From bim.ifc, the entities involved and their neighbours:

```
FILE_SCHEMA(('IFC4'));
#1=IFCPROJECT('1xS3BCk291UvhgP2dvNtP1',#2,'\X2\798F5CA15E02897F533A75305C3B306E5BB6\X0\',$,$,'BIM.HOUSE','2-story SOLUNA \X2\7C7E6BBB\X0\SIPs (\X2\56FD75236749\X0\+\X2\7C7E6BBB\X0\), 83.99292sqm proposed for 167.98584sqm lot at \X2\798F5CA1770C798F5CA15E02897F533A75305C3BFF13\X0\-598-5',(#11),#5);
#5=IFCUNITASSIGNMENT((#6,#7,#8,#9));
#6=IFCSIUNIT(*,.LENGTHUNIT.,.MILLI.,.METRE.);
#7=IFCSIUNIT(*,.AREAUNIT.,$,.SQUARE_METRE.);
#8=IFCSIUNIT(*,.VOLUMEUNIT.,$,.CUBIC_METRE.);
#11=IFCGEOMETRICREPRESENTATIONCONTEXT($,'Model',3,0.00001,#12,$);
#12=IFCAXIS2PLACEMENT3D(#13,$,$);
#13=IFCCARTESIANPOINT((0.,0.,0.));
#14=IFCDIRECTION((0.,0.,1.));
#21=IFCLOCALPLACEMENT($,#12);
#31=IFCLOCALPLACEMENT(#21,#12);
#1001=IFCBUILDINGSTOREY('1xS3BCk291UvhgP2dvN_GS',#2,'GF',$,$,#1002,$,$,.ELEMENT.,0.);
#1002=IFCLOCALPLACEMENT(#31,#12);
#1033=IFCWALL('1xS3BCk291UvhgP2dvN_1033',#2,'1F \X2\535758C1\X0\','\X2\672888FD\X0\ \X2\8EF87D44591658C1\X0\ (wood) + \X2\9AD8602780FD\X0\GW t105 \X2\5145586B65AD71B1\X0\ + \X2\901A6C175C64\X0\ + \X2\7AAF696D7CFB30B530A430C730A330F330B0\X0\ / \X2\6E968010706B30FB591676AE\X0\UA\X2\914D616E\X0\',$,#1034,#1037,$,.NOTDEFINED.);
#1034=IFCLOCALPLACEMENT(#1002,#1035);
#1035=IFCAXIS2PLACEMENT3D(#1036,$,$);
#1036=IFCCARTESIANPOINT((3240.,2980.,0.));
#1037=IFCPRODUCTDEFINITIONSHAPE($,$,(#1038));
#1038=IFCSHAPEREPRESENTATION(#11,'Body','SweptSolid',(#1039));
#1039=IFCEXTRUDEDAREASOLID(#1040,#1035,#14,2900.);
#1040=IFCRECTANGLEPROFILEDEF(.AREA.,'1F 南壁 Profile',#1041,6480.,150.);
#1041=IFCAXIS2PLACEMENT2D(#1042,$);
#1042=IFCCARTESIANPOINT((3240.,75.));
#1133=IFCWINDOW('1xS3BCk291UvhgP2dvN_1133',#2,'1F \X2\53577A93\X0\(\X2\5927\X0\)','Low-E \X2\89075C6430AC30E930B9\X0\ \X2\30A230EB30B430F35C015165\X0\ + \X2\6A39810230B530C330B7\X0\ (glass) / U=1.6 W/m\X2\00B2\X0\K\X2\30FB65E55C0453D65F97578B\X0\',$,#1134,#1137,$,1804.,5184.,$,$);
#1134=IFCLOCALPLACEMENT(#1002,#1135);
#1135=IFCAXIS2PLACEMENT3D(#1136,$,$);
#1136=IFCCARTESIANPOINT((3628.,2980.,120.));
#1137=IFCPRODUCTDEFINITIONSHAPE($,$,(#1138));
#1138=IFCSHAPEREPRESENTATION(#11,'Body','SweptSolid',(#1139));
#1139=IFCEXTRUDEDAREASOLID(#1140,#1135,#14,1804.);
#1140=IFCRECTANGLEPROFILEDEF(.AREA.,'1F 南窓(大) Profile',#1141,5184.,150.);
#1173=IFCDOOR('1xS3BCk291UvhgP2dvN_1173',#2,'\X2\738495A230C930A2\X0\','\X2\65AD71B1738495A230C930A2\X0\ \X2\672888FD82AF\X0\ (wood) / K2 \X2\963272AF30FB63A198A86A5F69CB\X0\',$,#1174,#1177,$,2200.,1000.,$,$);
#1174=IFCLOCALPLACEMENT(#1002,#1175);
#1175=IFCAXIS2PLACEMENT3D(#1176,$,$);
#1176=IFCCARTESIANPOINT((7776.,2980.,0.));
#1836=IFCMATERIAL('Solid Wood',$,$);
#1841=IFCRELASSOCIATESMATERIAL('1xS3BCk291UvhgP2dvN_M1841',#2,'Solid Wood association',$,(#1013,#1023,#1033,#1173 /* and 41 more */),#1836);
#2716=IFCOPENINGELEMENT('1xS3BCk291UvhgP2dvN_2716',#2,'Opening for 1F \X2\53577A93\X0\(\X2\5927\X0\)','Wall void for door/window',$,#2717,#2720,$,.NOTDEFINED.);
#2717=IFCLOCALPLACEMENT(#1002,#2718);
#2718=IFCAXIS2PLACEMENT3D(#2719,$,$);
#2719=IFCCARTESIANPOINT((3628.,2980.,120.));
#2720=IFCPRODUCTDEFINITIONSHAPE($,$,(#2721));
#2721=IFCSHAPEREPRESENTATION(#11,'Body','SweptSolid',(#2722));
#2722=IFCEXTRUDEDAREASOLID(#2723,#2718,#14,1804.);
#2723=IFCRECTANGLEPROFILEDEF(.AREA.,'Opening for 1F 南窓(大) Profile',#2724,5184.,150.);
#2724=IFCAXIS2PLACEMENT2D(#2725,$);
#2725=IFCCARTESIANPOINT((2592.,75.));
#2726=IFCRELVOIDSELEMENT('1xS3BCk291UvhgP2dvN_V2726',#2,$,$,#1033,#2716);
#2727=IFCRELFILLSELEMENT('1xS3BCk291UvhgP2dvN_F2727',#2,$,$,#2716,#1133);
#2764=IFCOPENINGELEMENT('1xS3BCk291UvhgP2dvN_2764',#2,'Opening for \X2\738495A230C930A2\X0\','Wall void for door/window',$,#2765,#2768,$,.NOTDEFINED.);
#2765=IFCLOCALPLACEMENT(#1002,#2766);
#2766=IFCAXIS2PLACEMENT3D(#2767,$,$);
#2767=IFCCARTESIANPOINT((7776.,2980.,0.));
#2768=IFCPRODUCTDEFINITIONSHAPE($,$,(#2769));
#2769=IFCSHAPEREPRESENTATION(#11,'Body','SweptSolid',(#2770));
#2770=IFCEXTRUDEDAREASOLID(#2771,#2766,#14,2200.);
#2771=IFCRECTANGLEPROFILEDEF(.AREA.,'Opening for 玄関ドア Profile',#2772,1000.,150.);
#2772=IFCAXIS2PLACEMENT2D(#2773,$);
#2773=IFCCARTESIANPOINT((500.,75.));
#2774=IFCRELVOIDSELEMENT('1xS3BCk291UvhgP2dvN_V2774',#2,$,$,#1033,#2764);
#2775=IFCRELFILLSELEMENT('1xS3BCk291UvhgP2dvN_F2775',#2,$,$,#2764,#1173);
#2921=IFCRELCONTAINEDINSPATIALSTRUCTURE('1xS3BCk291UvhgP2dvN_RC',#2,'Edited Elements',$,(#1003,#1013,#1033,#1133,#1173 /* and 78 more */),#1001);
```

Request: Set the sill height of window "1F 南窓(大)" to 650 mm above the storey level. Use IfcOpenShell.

```python
import numpy as np
import ifcopenshell
import ifcopenshell.api.geometry
import ifcopenshell.geom
import ifcopenshell.util.element
import ifcopenshell.util.placement
import ifcopenshell.util.shape
import ifcopenshell.util.unit

model = ifcopenshell.open("bim.ifc")
unit_scale = ifcopenshell.util.unit.calculate_unit_scale(model)

window = model.by_guid("1xS3BCk291UvhgP2dvN_1133")
opening = window.FillsVoids[0].RelatingOpeningElement
storey = ifcopenshell.util.element.get_container(window, ifc_class="IfcBuildingStorey")
level = ifcopenshell.util.placement.get_local_placement(storey.ObjectPlacement)[2, 3]

# The opening's origin need not be at the sill, so measure its lowest point.
shape = ifcopenshell.geom.create_shape(ifcopenshell.geom.settings(), opening)
bottom = ifcopenshell.util.shape.get_shape_bottom_elevation(shape, shape.geometry) / unit_scale
dz = level + 0.65 / unit_scale - bottom

shift = np.array([0.0, 0.0, dz])
# The window is not placed relative to its opening, so move both.
for product in (opening, window):
    matrix = ifcopenshell.util.placement.get_local_placement(product.ObjectPlacement)
    matrix[:3, 3] += shift
    ifcopenshell.api.geometry.edit_object_placement(model, product=product, matrix=matrix, is_si=False)

print(f"moved by {dz * unit_scale:+.3f} m")

model.write("bim-out.ifc")
```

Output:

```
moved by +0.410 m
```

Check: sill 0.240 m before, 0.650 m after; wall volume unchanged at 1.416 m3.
